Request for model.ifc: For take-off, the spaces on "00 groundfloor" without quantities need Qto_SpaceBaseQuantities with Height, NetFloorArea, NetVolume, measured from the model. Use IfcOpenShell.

First a look at what the model holds.

```python
import ifcopenshell
import ifcopenshell.util.element
import ifcopenshell.util.unit

model = ifcopenshell.open("model.ifc")
print(model.schema)
for unit_type in ("LENGTHUNIT", "AREAUNIT", "VOLUMEUNIT"):
    print(unit_type, ifcopenshell.util.unit.calculate_unit_scale(model, unit_type))
storey = next(s for s in model.by_type("IfcBuildingStorey") if s.Name == "00 groundfloor")
spaces = [e for e in ifcopenshell.util.element.get_decomposition(storey) if e.is_a("IfcSpace")]
for e in sorted(spaces, key=lambda e: e.id()):
    print(e.id(), e.is_a(), e.Name, list(ifcopenshell.util.element.get_psets(e, qtos_only=True)), sep=" | ")
```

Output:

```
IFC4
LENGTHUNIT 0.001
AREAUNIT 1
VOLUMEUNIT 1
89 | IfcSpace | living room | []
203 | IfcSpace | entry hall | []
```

```python
import ifcopenshell
import ifcopenshell.api.pset
import ifcopenshell.geom
import ifcopenshell.util.element
import ifcopenshell.util.shape
import ifcopenshell.util.unit

model = ifcopenshell.open("model.ifc")
unit_scale = ifcopenshell.util.unit.calculate_unit_scale(model)
area_scale = ifcopenshell.util.unit.calculate_unit_scale(model, "AREAUNIT")
volume_scale = ifcopenshell.util.unit.calculate_unit_scale(model, "VOLUMEUNIT")
settings = ifcopenshell.geom.settings()

storey = next(s for s in model.by_type("IfcBuildingStorey") if s.Name == "00 groundfloor")
spaces = [e for e in ifcopenshell.util.element.get_decomposition(storey) if e.is_a("IfcSpace")]

for e in sorted(spaces, key=lambda e: e.id()):
    if ifcopenshell.util.element.get_psets(e, qtos_only=True, should_inherit=False):
        continue
    # Geometry comes back in metres, in the element's own axes.
    shape = ifcopenshell.geom.create_shape(settings, e)
    values = {
        "Height": ifcopenshell.util.shape.get_z(shape.geometry) / unit_scale,
        "NetFloorArea": ifcopenshell.util.shape.get_footprint_area(shape.geometry) / area_scale,
        "NetVolume": ifcopenshell.util.shape.get_volume(shape.geometry) / volume_scale,
    }
    qto = ifcopenshell.api.pset.add_qto(model, product=e, name="Qto_SpaceBaseQuantities")
    ifcopenshell.api.pset.edit_qto(model, qto=qto, properties=values)
    print(e.id(), {k: round(v, 3) for k, v in values.items()})

model.write("model_v2.ifc")
```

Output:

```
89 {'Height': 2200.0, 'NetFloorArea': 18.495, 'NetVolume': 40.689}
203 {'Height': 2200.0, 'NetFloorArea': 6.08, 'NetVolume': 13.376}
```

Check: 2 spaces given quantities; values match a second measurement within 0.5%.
